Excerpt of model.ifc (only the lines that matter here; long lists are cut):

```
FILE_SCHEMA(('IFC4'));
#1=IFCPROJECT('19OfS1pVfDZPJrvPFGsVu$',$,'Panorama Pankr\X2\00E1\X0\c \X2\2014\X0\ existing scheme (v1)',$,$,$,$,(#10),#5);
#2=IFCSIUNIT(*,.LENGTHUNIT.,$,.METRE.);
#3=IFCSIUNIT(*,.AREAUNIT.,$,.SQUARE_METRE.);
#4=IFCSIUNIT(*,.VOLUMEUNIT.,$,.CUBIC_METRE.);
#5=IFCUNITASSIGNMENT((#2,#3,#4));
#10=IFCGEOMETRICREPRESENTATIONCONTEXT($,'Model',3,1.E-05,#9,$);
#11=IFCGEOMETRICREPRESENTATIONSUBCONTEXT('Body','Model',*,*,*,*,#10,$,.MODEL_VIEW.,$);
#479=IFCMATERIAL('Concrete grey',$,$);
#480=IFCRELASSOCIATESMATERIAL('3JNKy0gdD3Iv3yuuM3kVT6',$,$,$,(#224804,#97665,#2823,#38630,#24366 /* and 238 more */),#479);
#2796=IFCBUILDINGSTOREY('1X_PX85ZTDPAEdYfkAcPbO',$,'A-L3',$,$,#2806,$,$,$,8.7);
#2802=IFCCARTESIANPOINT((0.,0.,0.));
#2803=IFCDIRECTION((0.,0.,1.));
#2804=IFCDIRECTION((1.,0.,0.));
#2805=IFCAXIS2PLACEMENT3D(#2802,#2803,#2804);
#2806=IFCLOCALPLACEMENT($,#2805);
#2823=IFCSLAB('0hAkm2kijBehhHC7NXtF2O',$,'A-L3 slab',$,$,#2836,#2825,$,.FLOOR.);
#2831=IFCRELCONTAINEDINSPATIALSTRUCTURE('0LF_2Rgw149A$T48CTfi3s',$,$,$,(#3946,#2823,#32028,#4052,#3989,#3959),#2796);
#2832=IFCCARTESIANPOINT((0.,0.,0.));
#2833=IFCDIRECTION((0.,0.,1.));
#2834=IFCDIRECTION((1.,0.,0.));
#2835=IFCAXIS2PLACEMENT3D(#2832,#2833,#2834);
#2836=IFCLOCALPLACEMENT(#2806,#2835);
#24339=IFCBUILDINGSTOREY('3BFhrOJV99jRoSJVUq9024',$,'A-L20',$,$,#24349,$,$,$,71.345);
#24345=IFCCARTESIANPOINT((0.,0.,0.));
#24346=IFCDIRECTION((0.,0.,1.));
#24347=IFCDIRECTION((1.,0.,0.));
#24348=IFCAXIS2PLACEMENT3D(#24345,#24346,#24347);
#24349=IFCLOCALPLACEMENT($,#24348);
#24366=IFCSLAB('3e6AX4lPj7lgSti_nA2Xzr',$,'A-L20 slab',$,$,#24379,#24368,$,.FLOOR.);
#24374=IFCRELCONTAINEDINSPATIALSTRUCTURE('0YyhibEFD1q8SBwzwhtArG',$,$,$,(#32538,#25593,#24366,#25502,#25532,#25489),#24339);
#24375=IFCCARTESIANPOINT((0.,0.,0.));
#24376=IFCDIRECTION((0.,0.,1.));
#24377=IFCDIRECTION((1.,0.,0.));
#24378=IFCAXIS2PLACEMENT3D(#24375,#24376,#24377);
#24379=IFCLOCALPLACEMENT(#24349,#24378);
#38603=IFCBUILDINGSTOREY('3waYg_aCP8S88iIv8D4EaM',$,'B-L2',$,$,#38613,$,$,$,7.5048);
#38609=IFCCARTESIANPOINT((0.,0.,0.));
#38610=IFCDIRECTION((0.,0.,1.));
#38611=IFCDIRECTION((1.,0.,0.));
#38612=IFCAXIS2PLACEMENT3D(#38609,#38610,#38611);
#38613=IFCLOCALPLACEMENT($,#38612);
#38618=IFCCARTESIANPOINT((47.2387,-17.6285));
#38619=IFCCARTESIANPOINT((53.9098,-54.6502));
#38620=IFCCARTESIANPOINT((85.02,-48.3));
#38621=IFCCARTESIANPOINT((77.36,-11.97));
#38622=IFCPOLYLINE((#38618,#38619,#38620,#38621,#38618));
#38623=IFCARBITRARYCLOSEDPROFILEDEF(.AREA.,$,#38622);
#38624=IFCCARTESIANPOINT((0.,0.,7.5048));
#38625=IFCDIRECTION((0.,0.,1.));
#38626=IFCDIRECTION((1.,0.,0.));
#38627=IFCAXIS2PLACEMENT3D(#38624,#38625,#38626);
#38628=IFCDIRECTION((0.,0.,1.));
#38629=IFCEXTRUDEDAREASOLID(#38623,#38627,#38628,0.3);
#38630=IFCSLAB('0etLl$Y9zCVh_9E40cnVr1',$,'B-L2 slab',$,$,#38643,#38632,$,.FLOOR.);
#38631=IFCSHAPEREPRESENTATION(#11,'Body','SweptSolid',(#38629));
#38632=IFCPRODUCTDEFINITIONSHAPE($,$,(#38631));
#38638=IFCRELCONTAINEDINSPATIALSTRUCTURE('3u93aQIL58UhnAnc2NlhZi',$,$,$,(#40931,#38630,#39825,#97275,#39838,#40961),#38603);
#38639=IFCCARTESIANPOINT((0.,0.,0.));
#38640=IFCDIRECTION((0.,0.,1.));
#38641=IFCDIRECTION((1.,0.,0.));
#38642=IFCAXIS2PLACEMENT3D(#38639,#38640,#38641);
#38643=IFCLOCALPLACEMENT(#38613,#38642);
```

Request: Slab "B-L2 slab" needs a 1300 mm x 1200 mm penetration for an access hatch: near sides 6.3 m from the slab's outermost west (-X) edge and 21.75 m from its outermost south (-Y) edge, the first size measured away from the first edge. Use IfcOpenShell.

```python
import numpy as np
import ifcopenshell
import ifcopenshell.api.feature
import ifcopenshell.api.geometry
import ifcopenshell.api.root
import ifcopenshell.geom
import ifcopenshell.util.placement
import ifcopenshell.util.representation
import ifcopenshell.util.shape
import ifcopenshell.util.unit

model = ifcopenshell.open("model.ifc")
unit_scale = ifcopenshell.util.unit.calculate_unit_scale(model)
settings = ifcopenshell.geom.settings()


def volume(element):
    """Net volume in cubic metres, openings subtracted."""
    shape = ifcopenshell.geom.create_shape(settings, element)
    return ifcopenshell.util.shape.get_volume(shape.geometry)


slab = model.by_id(38630)
before = volume(slab)

# Extent in the slab's own axes, in metres. The edges named are its -X and -Y sides.
slab_shape = ifcopenshell.geom.create_shape(settings, slab)
vertices = ifcopenshell.util.shape.get_vertices(slab_shape.geometry)
x_min, y_min, bottom = vertices.min(axis=0)
top = vertices[:, 2].max()

opening = ifcopenshell.api.root.create_entity(model, ifc_class="IfcOpeningElement", name="Access hatch opening", predefined_type="OPENING")
context = ifcopenshell.util.representation.get_context(model, "Model", "Body", "MODEL_VIEW")
width, depth = 1.3, 1.2
outline = [(0.0, 0.0), (width, 0.0), (width, depth), (0.0, depth), (0.0, 0.0)]
# Overshoot both faces by 50 mm so the cut is clean.
shape = ifcopenshell.api.geometry.add_slab_representation(
    model, context=context, depth=top - bottom + 0.1, polyline=outline
)
ifcopenshell.api.geometry.assign_representation(model, product=opening, representation=shape)

matrix = ifcopenshell.util.placement.get_local_placement(slab.ObjectPlacement)
matrix[:, 3] = matrix @ np.append(np.array([x_min + 6.3, y_min + 21.75, bottom - 0.05]) / unit_scale, 1.0)
ifcopenshell.api.geometry.edit_object_placement(model, product=opening, matrix=matrix, is_si=False)
ifcopenshell.api.feature.add_feature(model, feature=opening, element=slab)

after = volume(slab)

print(f"slab volume {before:.3f} -> {after:.3f} m3")

model.write("model_rev.ifc")
```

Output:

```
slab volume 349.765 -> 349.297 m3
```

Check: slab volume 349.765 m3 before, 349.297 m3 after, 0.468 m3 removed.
